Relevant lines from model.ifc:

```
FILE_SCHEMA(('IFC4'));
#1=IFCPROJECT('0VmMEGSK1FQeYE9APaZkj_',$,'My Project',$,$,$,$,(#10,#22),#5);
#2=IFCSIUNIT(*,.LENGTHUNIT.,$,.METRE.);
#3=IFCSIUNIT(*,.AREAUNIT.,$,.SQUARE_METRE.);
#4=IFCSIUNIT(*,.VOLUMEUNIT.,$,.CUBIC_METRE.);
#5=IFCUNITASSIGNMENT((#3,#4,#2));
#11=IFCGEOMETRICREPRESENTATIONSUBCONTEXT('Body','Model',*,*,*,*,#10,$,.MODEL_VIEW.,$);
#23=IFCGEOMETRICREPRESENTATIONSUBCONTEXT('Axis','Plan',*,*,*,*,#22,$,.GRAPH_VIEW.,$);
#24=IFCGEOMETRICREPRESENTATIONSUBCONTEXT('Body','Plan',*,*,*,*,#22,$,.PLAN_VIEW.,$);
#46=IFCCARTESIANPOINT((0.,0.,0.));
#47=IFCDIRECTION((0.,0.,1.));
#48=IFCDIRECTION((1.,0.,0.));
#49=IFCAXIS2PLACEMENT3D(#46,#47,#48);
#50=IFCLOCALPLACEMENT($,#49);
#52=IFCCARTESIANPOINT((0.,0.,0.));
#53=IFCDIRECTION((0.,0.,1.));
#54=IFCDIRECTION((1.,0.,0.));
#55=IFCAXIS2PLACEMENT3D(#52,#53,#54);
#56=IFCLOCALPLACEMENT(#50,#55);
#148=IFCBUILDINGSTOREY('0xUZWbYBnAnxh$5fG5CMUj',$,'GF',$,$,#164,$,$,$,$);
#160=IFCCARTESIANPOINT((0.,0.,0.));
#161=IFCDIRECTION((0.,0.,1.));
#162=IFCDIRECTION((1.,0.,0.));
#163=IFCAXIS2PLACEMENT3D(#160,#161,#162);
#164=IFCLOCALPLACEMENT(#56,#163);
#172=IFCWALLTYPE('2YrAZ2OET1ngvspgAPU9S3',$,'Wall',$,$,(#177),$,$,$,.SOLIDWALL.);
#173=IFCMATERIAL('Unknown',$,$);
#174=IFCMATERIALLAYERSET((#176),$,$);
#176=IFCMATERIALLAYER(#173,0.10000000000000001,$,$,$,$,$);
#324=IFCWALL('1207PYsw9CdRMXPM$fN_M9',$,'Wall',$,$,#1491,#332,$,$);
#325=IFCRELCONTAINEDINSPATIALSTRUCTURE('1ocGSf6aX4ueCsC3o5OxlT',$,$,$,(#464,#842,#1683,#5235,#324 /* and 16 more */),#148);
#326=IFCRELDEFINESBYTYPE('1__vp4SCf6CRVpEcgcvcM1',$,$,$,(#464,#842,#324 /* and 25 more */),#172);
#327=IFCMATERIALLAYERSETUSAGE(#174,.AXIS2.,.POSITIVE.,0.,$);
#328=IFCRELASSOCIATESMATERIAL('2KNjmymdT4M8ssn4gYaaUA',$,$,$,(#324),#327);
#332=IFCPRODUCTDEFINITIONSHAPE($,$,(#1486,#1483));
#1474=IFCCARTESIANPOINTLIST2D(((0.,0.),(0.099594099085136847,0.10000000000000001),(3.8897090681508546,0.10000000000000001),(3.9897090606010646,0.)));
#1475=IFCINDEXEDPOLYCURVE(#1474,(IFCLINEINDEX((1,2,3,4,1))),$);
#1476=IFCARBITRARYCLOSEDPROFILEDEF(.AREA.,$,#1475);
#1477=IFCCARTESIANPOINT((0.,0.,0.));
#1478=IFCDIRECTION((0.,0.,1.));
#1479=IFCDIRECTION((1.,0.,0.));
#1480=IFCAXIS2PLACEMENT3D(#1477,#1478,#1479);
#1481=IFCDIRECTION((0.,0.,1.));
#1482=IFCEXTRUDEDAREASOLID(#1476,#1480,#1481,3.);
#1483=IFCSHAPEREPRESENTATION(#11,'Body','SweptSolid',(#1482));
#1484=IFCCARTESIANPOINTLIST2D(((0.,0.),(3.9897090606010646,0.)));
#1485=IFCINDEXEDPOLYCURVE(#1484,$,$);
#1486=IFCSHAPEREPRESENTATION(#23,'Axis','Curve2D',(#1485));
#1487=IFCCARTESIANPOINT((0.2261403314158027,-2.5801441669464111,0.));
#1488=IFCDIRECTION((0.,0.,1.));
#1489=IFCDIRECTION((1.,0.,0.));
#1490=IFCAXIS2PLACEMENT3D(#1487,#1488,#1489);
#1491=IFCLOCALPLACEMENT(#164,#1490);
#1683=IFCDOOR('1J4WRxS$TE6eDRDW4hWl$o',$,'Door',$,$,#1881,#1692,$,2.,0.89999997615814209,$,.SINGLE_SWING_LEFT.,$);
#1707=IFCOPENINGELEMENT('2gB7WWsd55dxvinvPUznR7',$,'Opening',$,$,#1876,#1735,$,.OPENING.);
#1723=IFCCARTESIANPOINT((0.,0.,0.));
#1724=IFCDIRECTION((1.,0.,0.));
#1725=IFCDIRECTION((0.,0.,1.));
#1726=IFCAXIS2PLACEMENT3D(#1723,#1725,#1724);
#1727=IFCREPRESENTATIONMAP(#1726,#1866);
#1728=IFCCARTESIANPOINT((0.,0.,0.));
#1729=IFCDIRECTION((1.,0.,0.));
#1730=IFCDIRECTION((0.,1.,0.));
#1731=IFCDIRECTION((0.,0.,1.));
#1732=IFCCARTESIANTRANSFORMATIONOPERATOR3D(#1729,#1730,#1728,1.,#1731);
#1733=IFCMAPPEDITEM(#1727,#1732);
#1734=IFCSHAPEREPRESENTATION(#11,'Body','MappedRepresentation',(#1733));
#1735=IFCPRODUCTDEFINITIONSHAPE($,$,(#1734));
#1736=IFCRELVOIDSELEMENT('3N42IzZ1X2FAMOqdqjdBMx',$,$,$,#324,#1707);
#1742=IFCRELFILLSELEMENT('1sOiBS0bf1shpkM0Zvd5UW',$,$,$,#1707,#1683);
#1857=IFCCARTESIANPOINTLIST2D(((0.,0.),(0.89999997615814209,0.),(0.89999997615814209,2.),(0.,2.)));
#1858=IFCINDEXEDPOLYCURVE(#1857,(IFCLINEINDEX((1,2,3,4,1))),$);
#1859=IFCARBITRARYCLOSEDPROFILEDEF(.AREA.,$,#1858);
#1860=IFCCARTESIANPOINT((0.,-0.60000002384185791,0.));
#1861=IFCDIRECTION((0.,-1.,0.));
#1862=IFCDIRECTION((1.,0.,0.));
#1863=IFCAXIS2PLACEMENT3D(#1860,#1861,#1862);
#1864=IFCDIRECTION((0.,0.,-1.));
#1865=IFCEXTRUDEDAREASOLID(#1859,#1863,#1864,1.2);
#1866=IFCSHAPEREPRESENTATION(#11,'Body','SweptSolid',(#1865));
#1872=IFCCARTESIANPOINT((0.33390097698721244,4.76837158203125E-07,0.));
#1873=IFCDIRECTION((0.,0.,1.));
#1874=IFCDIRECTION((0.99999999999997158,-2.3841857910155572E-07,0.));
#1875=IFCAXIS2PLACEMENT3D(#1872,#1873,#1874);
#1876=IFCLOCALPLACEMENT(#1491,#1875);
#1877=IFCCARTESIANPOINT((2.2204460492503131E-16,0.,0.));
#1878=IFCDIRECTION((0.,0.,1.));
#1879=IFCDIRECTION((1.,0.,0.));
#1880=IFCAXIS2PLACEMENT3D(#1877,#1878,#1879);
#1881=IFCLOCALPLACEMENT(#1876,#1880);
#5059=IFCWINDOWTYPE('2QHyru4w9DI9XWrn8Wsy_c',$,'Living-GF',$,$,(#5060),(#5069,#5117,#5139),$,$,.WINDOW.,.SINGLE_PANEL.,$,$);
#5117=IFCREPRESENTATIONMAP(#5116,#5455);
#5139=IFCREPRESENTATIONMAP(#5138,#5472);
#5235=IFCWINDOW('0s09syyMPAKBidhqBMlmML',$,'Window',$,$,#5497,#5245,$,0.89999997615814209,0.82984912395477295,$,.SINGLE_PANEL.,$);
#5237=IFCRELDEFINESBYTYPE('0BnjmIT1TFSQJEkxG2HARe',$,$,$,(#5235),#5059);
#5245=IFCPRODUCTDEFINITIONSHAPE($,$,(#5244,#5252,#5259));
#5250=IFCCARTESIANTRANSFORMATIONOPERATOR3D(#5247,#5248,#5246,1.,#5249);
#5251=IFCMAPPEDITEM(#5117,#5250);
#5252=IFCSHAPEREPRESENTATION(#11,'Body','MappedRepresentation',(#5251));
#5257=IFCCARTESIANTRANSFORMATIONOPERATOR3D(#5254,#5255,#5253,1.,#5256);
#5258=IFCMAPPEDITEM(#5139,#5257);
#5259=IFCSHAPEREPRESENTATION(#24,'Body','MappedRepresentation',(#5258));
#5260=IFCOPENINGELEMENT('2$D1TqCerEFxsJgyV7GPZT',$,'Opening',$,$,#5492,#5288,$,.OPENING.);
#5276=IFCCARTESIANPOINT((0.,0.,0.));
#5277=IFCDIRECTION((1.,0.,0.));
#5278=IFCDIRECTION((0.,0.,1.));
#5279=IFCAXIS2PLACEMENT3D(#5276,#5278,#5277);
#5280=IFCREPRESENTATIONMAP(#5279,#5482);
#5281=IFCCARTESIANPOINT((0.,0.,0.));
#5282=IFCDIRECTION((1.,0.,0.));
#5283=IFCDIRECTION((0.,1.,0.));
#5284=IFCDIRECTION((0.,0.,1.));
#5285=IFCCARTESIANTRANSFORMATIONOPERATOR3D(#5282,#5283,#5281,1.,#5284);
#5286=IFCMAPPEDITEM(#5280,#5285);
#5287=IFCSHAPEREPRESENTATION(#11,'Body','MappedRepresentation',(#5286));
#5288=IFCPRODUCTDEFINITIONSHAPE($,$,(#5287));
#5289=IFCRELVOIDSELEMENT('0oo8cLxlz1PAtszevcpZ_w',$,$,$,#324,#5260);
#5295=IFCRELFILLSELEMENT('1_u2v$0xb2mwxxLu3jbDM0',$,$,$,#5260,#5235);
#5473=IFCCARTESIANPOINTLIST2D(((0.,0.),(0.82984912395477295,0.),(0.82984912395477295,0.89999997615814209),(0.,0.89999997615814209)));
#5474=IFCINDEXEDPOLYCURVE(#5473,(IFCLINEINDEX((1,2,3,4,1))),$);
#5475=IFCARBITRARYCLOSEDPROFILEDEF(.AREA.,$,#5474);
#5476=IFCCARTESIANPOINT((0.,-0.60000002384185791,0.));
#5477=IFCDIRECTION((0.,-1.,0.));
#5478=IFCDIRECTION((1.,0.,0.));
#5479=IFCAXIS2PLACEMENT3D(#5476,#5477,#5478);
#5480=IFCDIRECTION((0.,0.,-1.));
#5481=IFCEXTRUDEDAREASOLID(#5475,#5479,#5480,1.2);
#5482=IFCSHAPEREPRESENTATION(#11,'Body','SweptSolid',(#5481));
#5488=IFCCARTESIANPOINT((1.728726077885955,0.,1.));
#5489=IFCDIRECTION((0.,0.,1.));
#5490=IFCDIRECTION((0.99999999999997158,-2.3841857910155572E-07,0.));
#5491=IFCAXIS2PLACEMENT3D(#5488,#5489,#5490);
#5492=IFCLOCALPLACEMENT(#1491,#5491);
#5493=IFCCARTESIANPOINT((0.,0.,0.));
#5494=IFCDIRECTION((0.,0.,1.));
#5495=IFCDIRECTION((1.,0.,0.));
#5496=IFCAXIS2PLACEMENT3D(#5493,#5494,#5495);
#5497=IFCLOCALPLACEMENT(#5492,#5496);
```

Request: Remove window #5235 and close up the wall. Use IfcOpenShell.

```python
import ifcopenshell
import ifcopenshell.api.feature
import ifcopenshell.api.root
import ifcopenshell.geom
import ifcopenshell.util.shape

model = ifcopenshell.open("model.ifc")
settings = ifcopenshell.geom.settings()


def volume(element):
    """Net volume in cubic metres, openings subtracted."""
    shape = ifcopenshell.geom.create_shape(settings, element)
    return ifcopenshell.util.shape.get_volume(shape.geometry)


window = model.by_id(5235)
opening = window.FillsVoids[0].RelatingOpeningElement
wall = opening.VoidsElements[0].RelatingBuildingElement
before = volume(wall)

ifcopenshell.api.root.remove_product(model, product=window)
ifcopenshell.api.feature.remove_feature(model, feature=opening)

after = volume(wall)

print(f"wall volume {before:.3f} -> {after:.3f} m3")

model.write("model_edited.ifc")
```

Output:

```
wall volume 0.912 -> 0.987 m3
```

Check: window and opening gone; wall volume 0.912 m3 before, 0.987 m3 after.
